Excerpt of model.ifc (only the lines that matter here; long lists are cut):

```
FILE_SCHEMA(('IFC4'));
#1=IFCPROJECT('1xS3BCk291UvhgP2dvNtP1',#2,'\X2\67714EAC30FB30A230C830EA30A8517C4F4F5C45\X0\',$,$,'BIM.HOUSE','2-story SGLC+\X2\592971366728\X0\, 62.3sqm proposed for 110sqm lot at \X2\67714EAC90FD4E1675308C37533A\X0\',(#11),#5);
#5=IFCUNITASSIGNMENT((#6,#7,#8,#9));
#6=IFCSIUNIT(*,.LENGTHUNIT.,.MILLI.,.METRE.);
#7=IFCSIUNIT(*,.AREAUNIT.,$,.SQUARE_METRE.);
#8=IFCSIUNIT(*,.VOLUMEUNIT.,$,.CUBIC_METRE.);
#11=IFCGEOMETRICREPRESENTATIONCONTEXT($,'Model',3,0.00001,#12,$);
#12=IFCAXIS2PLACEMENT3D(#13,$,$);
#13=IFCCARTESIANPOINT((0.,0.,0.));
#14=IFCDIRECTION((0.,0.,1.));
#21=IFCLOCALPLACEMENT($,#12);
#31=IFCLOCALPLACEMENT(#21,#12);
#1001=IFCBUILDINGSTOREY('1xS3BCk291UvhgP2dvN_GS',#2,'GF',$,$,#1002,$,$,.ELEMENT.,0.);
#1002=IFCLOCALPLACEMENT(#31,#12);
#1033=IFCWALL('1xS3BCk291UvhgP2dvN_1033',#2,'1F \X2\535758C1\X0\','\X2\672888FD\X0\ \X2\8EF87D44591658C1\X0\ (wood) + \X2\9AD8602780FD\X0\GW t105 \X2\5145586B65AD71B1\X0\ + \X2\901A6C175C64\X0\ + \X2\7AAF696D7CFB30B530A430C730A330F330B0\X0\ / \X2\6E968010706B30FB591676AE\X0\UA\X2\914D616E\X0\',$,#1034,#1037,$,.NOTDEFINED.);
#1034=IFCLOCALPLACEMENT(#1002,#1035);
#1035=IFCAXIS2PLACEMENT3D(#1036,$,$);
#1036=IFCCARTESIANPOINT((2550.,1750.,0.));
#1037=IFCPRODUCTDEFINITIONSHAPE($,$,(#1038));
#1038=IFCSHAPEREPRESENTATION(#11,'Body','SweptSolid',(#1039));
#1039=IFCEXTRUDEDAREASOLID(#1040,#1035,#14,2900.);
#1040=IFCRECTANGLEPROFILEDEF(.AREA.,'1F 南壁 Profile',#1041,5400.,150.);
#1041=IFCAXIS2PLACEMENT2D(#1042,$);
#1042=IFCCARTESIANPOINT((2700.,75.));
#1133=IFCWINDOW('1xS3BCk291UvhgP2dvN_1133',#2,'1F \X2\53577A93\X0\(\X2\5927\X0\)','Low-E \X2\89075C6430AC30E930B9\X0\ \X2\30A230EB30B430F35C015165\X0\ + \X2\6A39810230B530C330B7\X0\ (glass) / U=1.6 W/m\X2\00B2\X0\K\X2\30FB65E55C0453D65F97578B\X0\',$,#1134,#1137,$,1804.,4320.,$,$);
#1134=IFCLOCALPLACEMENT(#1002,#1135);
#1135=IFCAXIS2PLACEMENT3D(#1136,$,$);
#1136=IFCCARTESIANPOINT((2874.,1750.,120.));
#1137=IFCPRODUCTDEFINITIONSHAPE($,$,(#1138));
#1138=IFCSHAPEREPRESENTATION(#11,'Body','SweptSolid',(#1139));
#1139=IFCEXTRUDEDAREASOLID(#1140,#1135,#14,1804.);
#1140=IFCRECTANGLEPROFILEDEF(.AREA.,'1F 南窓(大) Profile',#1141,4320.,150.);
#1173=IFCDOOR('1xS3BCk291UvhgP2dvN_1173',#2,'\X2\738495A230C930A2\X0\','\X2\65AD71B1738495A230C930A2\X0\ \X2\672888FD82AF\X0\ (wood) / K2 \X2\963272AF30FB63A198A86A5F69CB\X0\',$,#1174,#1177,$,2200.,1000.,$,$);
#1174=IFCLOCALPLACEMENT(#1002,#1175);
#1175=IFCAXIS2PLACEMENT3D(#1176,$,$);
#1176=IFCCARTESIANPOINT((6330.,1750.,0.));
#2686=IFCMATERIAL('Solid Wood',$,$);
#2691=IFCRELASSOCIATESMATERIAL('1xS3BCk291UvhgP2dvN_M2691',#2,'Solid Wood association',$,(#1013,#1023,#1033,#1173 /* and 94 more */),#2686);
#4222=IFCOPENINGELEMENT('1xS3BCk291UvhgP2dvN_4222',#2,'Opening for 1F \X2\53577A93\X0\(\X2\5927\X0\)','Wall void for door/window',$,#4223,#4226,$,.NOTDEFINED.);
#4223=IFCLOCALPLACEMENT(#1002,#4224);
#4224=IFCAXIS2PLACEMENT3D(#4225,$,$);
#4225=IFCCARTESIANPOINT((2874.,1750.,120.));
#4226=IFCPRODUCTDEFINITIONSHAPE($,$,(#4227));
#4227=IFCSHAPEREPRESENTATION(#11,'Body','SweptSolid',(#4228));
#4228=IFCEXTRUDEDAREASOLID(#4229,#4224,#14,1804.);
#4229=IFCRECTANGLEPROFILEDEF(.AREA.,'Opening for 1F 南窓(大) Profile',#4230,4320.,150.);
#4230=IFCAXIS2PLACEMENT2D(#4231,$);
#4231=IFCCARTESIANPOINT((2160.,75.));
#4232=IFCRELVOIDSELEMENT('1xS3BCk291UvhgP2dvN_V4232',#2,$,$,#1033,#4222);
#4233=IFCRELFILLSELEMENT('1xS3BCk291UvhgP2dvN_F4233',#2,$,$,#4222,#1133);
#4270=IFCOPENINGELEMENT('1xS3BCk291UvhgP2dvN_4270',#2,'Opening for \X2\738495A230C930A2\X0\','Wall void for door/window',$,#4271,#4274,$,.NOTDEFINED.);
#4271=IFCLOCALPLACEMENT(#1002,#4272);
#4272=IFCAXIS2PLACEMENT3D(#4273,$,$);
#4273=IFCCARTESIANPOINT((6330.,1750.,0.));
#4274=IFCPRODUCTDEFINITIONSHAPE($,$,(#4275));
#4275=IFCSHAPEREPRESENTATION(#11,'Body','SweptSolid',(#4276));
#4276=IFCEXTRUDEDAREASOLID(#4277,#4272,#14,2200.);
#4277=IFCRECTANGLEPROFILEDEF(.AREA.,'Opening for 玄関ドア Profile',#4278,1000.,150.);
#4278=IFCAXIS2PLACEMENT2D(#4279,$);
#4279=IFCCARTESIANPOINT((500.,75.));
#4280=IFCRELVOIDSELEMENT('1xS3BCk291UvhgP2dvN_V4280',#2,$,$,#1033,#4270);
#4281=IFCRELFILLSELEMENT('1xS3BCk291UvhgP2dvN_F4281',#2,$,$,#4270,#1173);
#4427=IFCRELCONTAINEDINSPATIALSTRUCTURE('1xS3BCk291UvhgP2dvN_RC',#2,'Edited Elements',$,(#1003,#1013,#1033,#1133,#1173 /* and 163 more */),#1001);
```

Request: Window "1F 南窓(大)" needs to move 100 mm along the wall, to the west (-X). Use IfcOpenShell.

```python
import ifcopenshell
import ifcopenshell.api.geometry
import ifcopenshell.util.placement
import ifcopenshell.util.unit

model = ifcopenshell.open("model.ifc")
unit_scale = ifcopenshell.util.unit.calculate_unit_scale(model)

window = model.by_guid("1xS3BCk291UvhgP2dvN_1133")
opening = window.FillsVoids[0].RelatingOpeningElement
wall = opening.VoidsElements[0].RelatingBuildingElement

wall_matrix = ifcopenshell.util.placement.get_local_placement(wall.ObjectPlacement)
shift = wall_matrix[:3, 0] * -0.1 / unit_scale
before = ifcopenshell.util.placement.get_local_placement(window.ObjectPlacement)[:3, 3].copy()

# The window is not placed relative to its opening, so move both.
for product in (opening, window):
    matrix = ifcopenshell.util.placement.get_local_placement(product.ObjectPlacement)
    matrix[:3, 3] += shift
    ifcopenshell.api.geometry.edit_object_placement(model, product=product, matrix=matrix, is_si=False)

after = ifcopenshell.util.placement.get_local_placement(window.ObjectPlacement)[:3, 3]
print("window moved by", (after - before).round(3) + 0.0)

model.write("model-out.ifc")
```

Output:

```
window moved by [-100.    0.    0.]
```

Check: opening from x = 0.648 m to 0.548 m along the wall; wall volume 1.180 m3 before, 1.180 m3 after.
